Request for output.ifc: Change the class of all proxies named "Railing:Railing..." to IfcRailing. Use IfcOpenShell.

First a look at what the model holds.

```python
import re

import ifcopenshell

model = ifcopenshell.open("output.ifc")
print(model.schema)
seen = {}
for e in model.by_type("IfcBuildingElementProxy"):
    name = re.sub(r":\d+(:\d+)?$", "", e.Name or "")  # drop the element id that some exporters append
    seen[name] = seen.get(name, 0) + 1
for name, count in sorted(seen.items()):
    print(count, "x", name)
```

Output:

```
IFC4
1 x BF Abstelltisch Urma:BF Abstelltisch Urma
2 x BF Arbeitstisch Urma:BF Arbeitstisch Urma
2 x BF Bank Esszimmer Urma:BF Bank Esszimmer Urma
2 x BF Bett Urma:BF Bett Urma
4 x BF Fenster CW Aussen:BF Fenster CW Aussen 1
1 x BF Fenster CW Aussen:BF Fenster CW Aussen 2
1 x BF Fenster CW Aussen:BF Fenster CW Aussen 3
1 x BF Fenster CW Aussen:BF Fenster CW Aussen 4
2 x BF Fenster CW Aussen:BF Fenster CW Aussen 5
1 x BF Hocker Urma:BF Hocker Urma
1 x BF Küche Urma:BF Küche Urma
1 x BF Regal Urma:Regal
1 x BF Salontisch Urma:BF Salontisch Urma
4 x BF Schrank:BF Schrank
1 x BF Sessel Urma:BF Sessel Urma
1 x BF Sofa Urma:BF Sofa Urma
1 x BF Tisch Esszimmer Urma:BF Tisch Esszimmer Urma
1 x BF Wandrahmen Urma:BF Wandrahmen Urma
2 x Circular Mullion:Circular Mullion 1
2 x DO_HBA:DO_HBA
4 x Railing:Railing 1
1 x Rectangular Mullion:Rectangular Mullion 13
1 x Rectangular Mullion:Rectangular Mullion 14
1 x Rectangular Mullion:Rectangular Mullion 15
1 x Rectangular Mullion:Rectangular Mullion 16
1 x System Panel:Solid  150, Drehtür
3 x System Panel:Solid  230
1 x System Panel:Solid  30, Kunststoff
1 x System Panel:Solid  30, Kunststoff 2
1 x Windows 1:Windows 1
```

```python
import ifcopenshell
import ifcopenshell.api.root

model = ifcopenshell.open("output.ifc")

proxies = [e.id() for e in model.by_type("IfcBuildingElementProxy") if (e.Name or "").startswith("Railing:Railing")]
for step_id in proxies:
    proxy = model.by_id(step_id)
    ifcopenshell.api.root.reassign_class(model, product=proxy, ifc_class="IfcRailing")

print(sum(model.by_id(i).is_a("IfcRailing") for i in proxies), "reclassified")

model.write("output_rev.ifc")
```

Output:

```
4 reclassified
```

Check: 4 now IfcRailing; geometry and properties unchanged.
